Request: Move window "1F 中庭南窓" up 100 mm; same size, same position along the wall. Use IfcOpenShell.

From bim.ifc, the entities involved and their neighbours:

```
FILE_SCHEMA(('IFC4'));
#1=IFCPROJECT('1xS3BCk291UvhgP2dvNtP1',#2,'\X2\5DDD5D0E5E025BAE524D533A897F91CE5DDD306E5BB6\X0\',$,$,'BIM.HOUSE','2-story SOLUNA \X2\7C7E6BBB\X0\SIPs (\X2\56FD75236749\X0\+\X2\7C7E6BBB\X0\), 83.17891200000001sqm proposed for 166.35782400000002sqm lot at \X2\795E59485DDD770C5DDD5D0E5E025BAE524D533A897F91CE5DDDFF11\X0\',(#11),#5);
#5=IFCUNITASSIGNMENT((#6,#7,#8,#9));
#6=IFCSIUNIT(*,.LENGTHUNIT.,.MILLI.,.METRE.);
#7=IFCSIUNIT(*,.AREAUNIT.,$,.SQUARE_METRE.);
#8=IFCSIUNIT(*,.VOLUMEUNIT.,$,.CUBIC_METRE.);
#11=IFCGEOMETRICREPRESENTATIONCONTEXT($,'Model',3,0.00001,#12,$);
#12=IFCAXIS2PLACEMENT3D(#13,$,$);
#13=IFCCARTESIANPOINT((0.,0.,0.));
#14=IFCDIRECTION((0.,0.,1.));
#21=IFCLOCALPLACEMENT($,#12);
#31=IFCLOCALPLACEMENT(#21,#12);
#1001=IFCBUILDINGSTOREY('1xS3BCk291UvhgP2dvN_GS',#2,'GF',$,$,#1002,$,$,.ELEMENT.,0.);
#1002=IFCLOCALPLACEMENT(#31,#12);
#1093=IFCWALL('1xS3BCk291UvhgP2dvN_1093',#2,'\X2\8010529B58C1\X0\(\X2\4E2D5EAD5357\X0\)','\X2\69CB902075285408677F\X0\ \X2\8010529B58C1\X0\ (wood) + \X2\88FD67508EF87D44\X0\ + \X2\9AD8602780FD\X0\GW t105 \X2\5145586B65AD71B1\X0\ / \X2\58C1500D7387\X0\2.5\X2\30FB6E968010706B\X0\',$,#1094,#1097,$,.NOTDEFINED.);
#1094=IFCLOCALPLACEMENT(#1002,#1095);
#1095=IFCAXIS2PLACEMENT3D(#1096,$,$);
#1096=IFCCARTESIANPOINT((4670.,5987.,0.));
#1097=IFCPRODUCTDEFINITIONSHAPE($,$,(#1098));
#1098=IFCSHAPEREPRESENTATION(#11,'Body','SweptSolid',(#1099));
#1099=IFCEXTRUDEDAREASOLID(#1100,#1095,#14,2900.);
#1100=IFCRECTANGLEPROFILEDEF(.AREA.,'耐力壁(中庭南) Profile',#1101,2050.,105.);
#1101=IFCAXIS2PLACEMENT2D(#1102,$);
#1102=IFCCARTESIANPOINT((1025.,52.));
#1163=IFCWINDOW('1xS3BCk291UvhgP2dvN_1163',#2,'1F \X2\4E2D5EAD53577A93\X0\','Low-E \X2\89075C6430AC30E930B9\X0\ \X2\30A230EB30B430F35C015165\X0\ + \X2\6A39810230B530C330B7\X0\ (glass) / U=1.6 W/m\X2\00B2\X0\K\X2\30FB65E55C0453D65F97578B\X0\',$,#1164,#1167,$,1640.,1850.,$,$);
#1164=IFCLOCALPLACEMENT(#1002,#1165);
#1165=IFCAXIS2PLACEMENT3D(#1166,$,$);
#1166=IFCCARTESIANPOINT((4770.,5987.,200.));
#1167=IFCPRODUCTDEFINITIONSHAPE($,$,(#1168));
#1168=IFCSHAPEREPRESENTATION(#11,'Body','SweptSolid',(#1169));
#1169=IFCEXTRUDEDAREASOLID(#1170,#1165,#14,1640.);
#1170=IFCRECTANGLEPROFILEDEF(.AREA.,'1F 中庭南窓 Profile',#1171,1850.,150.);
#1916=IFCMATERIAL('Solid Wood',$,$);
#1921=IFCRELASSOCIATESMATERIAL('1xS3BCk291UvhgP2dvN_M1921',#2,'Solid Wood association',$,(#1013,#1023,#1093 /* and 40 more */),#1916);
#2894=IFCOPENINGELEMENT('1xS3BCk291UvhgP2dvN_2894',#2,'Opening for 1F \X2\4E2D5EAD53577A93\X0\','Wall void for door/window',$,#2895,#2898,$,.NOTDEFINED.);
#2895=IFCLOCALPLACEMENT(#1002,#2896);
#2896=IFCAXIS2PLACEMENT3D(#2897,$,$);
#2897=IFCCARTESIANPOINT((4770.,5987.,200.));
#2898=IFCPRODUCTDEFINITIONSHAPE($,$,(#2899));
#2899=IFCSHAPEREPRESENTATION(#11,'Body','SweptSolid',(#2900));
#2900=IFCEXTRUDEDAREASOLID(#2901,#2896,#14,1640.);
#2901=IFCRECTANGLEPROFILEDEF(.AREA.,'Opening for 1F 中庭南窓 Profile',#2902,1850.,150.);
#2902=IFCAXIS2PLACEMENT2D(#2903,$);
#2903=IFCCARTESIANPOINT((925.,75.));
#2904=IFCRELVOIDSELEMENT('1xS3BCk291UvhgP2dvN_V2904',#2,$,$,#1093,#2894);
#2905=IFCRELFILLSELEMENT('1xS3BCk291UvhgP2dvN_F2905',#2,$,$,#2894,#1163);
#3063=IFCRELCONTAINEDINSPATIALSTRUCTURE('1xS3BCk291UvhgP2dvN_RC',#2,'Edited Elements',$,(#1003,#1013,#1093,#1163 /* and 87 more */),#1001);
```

```python
import numpy as np
import ifcopenshell
import ifcopenshell.api.geometry
import ifcopenshell.util.placement
import ifcopenshell.util.unit

model = ifcopenshell.open("bim.ifc")
unit_scale = ifcopenshell.util.unit.calculate_unit_scale(model)

window = model.by_guid("1xS3BCk291UvhgP2dvN_1163")
opening = window.FillsVoids[0].RelatingOpeningElement
dz = 0.1 / unit_scale

shift = np.array([0.0, 0.0, dz])
# The window is not placed relative to its opening, so move both.
for product in (opening, window):
    matrix = ifcopenshell.util.placement.get_local_placement(product.ObjectPlacement)
    matrix[:3, 3] += shift
    ifcopenshell.api.geometry.edit_object_placement(model, product=product, matrix=matrix, is_si=False)

print(f"moved by {dz * unit_scale:+.3f} m")

model.write("bim_edited.ifc")
```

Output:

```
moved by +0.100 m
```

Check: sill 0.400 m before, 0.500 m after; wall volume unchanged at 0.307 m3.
